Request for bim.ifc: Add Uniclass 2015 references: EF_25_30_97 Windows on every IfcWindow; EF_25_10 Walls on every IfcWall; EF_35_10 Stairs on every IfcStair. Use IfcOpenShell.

First a look at what the model holds.

```python
import ifcopenshell

model = ifcopenshell.open("bim.ifc")
print(model.schema)
print("classifications:", [c.Name for c in model.by_type("IfcClassification")])
for ifc_class in ("IfcDoor", "IfcRoof", "IfcStair", "IfcWall", "IfcWindow"):
    print(ifc_class, len(model.by_type(ifc_class)))
```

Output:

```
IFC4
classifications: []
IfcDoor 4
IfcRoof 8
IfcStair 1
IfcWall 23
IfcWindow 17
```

```python
import ifcopenshell
import ifcopenshell.api.classification

model = ifcopenshell.open("bim.ifc")

system = ifcopenshell.api.classification.add_classification(model, classification="Uniclass 2015")

codes = {
    "IfcWindow": ("EF_25_30_97", "Windows"),
    "IfcWall": ("EF_25_10", "Walls"),
    "IfcStair": ("EF_35_10", "Stairs"),
}
for ifc_class, (code, name) in codes.items():
    products = model.by_type(ifc_class)
    ifcopenshell.api.classification.add_reference(
        model, products=products, classification=system, identification=code, name=name
    )
    print(code, len(products))

model.write("bim_v2.ifc")
```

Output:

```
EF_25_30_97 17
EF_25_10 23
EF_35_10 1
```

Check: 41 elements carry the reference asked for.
